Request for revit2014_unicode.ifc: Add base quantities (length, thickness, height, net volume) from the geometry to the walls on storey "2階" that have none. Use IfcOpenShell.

First a look at what the model holds.

```python
import ifcopenshell
import ifcopenshell.util.element
import ifcopenshell.util.unit

model = ifcopenshell.open("revit2014_unicode.ifc")
print(model.schema)
for unit_type in ("LENGTHUNIT", "AREAUNIT", "VOLUMEUNIT"):
    print(unit_type, ifcopenshell.util.unit.calculate_unit_scale(model, unit_type))
storey = next(s for s in model.by_type("IfcBuildingStorey") if s.Name == "2階")
walls = [e for e in ifcopenshell.util.element.get_decomposition(storey) if e.is_a("IfcWall")]
for e in sorted(walls, key=lambda e: e.id()):
    print(e.id(), e.is_a(), e.Name, list(ifcopenshell.util.element.get_psets(e, qtos_only=True)), sep=" | ")
```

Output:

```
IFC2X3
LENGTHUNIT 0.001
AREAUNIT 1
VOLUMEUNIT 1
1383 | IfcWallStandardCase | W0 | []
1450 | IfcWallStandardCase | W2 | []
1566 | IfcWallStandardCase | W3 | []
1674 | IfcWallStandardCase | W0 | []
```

```python
import ifcopenshell
import ifcopenshell.api.pset
import ifcopenshell.geom
import ifcopenshell.util.element
import ifcopenshell.util.shape
import ifcopenshell.util.unit

model = ifcopenshell.open("revit2014_unicode.ifc")
unit_scale = ifcopenshell.util.unit.calculate_unit_scale(model)
volume_scale = ifcopenshell.util.unit.calculate_unit_scale(model, "VOLUMEUNIT")
settings = ifcopenshell.geom.settings()

storey = next(s for s in model.by_type("IfcBuildingStorey") if s.Name == "2階")
walls = [e for e in ifcopenshell.util.element.get_decomposition(storey) if e.is_a("IfcWall")]

for e in sorted(walls, key=lambda e: e.id()):
    if ifcopenshell.util.element.get_psets(e, qtos_only=True, should_inherit=False):
        continue
    # Geometry comes back in metres, in the element's own axes.
    shape = ifcopenshell.geom.create_shape(settings, e)
    values = {
        "Length": ifcopenshell.util.shape.get_x(shape.geometry) / unit_scale,
        "Width": ifcopenshell.util.shape.get_y(shape.geometry) / unit_scale,
        "Height": ifcopenshell.util.shape.get_z(shape.geometry) / unit_scale,
        "NetVolume": ifcopenshell.util.shape.get_volume(shape.geometry) / volume_scale,
    }
    qto = ifcopenshell.api.pset.add_qto(model, product=e, name="BaseQuantities")
    ifcopenshell.api.pset.edit_qto(model, qto=qto, properties=values)
    print(e.id(), {k: round(v, 3) for k, v in values.items()})

model.write("revit2014_unicode_v2.ifc")
```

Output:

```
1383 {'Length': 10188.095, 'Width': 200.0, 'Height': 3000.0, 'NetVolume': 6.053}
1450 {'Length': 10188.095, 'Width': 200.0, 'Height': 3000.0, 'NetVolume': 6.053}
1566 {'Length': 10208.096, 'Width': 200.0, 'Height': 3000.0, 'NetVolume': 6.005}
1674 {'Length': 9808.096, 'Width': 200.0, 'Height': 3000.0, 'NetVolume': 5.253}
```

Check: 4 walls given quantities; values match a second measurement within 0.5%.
